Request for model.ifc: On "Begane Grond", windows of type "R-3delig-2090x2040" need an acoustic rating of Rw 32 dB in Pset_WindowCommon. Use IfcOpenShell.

First a look at what the model holds.

```python
import ifcopenshell
import ifcopenshell.util.element

model = ifcopenshell.open("model.ifc")
print(model.schema)
storey = next(s for s in model.by_type("IfcBuildingStorey") if s.Name == "Begane Grond")
windows = [e for e in ifcopenshell.util.element.get_decomposition(storey) if e.is_a("IfcWindow")]
seen = {}
for e in windows:
    element_type = ifcopenshell.util.element.get_type(e)
    key = (element_type.Name if element_type != e and element_type else None, ifcopenshell.util.element.get_pset(e, "Pset_WindowCommon", "AcousticRating"))
    seen[key] = seen.get(key, 0) + 1
for (name, value), count in sorted(seen.items(), key=str):
    print(count, "x", name, "|", value)
```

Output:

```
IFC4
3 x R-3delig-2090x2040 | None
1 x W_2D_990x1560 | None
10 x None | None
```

```python
import ifcopenshell
import ifcopenshell.api.pset
import ifcopenshell.util.element

model = ifcopenshell.open("model.ifc")

storey = next(s for s in model.by_type("IfcBuildingStorey") if s.Name == "Begane Grond")
windows = [e for e in ifcopenshell.util.element.get_decomposition(storey) if e.is_a("IfcWindow")]

count = 0
for e in windows:
    element_type = ifcopenshell.util.element.get_type(e)
    if element_type in (None, e) or element_type.Name != "R-3delig-2090x2040":
        continue
    # add_pset returns the element's existing set when there is one.
    pset = ifcopenshell.api.pset.add_pset(model, product=e, name="Pset_WindowCommon")
    ifcopenshell.api.pset.edit_pset(model, pset=pset, properties={"AcousticRating": "Rw 32 dB"})
    count += 1

print(count, "windows updated")

model.write("model_rev.ifc")
```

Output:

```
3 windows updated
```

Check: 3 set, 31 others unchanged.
